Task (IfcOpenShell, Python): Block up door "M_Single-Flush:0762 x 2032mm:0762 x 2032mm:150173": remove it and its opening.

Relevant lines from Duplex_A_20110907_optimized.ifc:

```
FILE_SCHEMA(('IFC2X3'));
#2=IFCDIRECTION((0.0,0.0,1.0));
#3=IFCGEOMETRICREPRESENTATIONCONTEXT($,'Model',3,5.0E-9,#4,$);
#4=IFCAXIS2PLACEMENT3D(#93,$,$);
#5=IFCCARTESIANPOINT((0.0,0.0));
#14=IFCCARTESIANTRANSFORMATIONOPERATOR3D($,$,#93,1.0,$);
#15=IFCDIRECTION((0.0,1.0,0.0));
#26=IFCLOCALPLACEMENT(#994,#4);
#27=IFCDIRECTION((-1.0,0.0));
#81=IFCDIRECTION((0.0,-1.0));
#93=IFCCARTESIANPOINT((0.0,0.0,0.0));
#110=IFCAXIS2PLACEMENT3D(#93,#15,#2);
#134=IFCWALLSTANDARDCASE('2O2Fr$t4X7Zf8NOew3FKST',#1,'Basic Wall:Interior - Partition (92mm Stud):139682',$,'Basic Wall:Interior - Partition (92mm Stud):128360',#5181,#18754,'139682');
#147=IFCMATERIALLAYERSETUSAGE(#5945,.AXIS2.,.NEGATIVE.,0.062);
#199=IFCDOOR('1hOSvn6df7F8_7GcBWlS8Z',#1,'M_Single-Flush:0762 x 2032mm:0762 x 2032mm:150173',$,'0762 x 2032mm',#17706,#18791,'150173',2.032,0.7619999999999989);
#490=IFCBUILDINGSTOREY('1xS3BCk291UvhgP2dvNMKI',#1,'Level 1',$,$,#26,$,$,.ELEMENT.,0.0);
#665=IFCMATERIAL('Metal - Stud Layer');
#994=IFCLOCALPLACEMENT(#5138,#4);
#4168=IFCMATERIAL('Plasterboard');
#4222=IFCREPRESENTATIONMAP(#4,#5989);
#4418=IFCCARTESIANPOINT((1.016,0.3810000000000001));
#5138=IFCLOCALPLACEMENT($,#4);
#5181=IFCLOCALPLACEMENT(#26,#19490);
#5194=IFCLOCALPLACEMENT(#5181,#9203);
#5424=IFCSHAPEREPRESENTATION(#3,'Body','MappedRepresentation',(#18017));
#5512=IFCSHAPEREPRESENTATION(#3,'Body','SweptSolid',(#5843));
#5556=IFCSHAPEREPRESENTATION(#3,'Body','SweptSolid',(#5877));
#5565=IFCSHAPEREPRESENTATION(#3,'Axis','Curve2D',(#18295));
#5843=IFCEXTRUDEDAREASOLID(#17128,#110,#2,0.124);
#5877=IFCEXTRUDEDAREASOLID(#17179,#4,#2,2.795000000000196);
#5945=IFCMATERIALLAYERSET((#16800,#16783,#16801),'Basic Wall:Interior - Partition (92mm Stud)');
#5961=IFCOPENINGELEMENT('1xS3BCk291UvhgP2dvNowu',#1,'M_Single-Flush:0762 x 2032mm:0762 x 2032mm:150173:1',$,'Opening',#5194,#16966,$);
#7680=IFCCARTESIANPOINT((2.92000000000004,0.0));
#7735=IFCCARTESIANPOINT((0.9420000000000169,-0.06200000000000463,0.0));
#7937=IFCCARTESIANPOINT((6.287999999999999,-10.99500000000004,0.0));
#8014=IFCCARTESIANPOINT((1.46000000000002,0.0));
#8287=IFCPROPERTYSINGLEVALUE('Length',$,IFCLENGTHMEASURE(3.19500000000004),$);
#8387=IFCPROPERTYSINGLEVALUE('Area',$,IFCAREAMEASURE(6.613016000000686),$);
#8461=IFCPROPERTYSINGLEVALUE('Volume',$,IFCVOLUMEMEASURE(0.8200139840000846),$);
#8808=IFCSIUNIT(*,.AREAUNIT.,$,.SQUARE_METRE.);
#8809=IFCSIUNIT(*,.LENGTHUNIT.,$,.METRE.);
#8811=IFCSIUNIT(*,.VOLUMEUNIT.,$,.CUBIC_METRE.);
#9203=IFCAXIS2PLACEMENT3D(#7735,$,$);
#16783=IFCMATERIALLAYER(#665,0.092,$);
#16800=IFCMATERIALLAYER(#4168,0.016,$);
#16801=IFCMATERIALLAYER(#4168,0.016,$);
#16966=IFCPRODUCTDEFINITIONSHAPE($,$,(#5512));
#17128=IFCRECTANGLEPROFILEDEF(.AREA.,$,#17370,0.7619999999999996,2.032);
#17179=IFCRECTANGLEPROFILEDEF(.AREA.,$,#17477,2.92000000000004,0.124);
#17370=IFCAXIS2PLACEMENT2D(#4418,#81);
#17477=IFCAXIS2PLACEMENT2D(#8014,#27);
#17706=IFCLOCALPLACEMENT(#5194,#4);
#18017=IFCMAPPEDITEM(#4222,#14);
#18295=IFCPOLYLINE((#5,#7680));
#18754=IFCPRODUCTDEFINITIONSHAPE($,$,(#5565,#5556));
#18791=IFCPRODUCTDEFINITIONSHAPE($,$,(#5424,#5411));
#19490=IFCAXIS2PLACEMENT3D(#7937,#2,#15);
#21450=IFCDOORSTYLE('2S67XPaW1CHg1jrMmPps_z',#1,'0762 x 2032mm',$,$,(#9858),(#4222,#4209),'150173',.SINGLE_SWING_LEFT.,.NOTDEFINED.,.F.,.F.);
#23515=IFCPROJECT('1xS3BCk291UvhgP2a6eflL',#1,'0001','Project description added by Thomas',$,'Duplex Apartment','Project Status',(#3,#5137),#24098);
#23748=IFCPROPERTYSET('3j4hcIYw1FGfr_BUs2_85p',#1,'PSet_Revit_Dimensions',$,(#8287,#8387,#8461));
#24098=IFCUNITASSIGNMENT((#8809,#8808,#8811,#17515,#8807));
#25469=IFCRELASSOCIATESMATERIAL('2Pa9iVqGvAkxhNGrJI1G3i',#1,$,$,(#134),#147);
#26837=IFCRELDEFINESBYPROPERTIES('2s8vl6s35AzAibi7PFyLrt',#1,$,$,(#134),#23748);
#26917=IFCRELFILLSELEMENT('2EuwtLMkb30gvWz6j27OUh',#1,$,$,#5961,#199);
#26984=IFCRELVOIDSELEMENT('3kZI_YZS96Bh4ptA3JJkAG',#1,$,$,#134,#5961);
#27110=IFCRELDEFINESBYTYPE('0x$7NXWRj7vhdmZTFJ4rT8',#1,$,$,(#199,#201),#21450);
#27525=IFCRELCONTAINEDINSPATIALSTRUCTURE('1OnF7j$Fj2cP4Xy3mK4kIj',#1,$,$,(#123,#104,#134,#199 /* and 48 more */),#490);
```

```python
import ifcopenshell
import ifcopenshell.api.feature
import ifcopenshell.api.pset
import ifcopenshell.api.root
import ifcopenshell.geom
import ifcopenshell.util.element
import ifcopenshell.util.shape
import ifcopenshell.util.unit

model = ifcopenshell.open("Duplex_A_20110907_optimized.ifc")
area_scale = ifcopenshell.util.unit.calculate_unit_scale(model, "AREAUNIT")
volume_scale = ifcopenshell.util.unit.calculate_unit_scale(model, "VOLUMEUNIT")
settings = ifcopenshell.geom.settings()


def volume(element):
    """Net volume in cubic metres, openings subtracted."""
    shape = ifcopenshell.geom.create_shape(settings, element)
    return ifcopenshell.util.shape.get_volume(shape.geometry)


door = model.by_id(199)
opening = door.FillsVoids[0].RelatingOpeningElement
wall = opening.VoidsElements[0].RelatingBuildingElement
before = volume(wall)

ifcopenshell.api.root.remove_product(model, product=door)
ifcopenshell.api.feature.remove_feature(model, feature=opening)

after = volume(wall)
thickness = 0.124  # wall thickness in metres

# Update the wall's stored quantities.
pset = model.by_id(ifcopenshell.util.element.get_pset(wall, "PSet_Revit_Dimensions", should_inherit=False)["id"])
ifcopenshell.api.pset.edit_pset(model, pset=pset, properties={
    "Area": model.create_entity("IfcAreaMeasure", after / thickness / area_scale),
    "Volume": model.create_entity("IfcVolumeMeasure", after / volume_scale),
})

print(f"wall volume {before:.3f} -> {after:.3f} m3")

model.write("Duplex_A_20110907_optimized-out.ifc")
```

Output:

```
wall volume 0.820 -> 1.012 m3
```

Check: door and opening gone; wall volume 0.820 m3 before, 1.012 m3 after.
